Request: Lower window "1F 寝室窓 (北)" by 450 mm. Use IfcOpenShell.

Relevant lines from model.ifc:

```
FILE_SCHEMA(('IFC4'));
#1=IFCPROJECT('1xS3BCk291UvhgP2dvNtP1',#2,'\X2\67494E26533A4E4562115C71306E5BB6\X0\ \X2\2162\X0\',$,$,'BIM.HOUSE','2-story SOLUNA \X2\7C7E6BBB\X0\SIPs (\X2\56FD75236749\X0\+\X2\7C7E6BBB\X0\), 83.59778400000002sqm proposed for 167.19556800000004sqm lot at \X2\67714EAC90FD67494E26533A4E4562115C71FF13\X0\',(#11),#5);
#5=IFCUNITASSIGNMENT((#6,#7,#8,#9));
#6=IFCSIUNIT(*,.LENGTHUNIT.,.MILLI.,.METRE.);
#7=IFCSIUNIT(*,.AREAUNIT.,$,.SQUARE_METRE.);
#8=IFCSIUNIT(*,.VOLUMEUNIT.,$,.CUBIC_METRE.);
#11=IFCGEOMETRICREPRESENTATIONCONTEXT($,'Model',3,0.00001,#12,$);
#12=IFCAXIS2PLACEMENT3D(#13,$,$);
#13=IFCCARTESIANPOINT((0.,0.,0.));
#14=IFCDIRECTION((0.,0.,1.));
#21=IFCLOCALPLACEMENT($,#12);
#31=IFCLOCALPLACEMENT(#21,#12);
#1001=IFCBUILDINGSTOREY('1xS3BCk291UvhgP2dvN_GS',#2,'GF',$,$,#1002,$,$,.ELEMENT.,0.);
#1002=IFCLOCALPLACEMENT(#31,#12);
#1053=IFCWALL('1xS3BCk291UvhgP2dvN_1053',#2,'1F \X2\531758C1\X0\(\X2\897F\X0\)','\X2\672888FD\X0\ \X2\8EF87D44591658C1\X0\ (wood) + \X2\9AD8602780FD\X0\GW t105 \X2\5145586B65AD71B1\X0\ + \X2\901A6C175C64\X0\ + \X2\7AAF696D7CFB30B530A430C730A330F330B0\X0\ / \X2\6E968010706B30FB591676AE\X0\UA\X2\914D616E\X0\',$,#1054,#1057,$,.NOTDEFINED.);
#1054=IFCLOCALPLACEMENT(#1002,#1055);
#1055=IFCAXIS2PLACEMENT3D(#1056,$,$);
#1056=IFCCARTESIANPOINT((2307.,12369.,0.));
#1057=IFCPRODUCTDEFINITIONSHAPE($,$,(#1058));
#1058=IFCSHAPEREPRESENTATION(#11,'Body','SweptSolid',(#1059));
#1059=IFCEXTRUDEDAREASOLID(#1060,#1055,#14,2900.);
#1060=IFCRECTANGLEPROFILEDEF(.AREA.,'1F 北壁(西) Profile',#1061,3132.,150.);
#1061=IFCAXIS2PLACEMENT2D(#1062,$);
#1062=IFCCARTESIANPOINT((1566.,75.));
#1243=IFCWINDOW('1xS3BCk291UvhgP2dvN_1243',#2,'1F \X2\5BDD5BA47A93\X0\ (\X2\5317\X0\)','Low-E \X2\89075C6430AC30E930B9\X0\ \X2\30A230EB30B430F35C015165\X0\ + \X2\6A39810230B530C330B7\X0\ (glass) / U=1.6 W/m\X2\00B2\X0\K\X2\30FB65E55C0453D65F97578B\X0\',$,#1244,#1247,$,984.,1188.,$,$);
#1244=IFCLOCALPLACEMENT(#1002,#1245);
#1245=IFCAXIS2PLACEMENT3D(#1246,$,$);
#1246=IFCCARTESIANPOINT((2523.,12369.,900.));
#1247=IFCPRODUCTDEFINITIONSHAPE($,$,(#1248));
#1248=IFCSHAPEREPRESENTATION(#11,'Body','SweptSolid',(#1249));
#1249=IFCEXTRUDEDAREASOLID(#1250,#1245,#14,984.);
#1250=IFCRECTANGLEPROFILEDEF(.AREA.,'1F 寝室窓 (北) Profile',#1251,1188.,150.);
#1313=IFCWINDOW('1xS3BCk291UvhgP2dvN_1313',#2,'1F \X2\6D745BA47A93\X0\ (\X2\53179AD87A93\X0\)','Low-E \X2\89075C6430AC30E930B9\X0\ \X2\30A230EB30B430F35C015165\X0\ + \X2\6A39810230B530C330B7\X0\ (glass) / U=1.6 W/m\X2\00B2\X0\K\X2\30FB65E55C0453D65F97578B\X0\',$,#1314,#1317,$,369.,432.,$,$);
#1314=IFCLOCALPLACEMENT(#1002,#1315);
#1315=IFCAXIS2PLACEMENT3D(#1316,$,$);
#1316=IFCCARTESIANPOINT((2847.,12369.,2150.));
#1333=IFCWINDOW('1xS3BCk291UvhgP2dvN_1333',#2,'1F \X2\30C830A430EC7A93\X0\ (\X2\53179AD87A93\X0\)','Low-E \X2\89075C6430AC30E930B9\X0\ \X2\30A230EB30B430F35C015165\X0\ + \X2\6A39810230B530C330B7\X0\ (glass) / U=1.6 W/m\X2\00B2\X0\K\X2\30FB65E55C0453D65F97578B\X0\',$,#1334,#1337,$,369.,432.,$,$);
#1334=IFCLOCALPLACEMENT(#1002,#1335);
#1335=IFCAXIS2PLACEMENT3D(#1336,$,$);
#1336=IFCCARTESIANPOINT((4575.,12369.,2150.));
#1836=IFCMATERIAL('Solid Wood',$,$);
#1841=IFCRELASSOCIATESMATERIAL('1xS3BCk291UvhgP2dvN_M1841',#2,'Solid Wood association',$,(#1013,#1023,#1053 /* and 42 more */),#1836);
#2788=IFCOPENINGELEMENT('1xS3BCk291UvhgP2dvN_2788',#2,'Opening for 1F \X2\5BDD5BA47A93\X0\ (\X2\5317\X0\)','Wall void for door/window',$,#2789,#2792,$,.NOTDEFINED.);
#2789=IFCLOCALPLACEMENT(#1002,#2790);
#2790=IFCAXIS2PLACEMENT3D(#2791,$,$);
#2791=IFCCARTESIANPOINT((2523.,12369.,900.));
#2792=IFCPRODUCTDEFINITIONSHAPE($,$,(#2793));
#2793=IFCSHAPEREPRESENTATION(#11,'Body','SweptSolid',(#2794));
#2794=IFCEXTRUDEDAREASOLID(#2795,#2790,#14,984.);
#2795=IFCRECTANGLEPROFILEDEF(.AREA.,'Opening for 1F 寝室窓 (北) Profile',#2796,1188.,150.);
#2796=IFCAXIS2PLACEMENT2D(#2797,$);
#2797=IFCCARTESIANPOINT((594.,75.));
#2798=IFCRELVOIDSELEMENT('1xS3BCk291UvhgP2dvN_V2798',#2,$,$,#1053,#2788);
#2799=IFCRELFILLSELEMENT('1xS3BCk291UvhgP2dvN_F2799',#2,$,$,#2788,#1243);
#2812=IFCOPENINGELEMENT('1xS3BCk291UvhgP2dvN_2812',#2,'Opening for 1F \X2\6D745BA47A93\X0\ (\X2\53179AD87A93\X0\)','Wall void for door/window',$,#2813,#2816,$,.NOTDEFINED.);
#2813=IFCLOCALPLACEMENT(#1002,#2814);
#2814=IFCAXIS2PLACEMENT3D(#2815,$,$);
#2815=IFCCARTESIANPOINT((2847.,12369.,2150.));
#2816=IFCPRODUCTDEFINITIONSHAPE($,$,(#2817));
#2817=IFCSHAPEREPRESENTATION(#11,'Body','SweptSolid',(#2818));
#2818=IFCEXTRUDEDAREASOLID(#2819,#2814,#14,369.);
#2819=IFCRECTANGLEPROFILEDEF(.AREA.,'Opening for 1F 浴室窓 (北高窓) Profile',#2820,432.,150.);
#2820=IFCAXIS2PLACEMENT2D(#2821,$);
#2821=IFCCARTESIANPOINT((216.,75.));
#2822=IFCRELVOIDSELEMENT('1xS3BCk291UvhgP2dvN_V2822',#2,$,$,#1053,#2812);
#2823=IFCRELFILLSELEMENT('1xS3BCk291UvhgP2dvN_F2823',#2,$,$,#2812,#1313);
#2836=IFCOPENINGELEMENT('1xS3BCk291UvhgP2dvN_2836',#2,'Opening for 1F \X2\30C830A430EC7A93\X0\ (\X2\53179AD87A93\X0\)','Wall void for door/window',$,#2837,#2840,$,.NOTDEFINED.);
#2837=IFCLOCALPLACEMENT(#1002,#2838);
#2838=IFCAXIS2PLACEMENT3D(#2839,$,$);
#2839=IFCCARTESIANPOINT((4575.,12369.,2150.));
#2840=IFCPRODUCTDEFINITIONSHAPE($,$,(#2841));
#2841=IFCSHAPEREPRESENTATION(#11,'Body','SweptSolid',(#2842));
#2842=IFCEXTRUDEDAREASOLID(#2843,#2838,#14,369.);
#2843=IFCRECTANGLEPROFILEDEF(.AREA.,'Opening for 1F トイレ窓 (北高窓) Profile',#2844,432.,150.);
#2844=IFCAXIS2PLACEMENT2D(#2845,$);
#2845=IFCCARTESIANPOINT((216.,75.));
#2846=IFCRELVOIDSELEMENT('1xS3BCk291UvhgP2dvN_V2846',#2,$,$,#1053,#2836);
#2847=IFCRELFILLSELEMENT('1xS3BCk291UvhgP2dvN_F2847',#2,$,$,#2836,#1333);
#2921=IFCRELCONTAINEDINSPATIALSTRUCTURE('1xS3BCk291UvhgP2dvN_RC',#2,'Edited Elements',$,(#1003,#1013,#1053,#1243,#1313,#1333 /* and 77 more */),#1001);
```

```python
import numpy as np
import ifcopenshell
import ifcopenshell.api.geometry
import ifcopenshell.util.placement
import ifcopenshell.util.unit

model = ifcopenshell.open("model.ifc")
unit_scale = ifcopenshell.util.unit.calculate_unit_scale(model)

window = model.by_id(1243)
opening = window.FillsVoids[0].RelatingOpeningElement
dz = -450.0

shift = np.array([0.0, 0.0, dz])
# The window is not placed relative to its opening, so move both.
for product in (opening, window):
    matrix = ifcopenshell.util.placement.get_local_placement(product.ObjectPlacement)
    matrix[:3, 3] += shift
    ifcopenshell.api.geometry.edit_object_placement(model, product=product, matrix=matrix, is_si=False)

print(f"moved by {dz * unit_scale:+.3f} m")

model.write("model_rev.ifc")
```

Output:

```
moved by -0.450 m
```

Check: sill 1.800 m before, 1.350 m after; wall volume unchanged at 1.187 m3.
